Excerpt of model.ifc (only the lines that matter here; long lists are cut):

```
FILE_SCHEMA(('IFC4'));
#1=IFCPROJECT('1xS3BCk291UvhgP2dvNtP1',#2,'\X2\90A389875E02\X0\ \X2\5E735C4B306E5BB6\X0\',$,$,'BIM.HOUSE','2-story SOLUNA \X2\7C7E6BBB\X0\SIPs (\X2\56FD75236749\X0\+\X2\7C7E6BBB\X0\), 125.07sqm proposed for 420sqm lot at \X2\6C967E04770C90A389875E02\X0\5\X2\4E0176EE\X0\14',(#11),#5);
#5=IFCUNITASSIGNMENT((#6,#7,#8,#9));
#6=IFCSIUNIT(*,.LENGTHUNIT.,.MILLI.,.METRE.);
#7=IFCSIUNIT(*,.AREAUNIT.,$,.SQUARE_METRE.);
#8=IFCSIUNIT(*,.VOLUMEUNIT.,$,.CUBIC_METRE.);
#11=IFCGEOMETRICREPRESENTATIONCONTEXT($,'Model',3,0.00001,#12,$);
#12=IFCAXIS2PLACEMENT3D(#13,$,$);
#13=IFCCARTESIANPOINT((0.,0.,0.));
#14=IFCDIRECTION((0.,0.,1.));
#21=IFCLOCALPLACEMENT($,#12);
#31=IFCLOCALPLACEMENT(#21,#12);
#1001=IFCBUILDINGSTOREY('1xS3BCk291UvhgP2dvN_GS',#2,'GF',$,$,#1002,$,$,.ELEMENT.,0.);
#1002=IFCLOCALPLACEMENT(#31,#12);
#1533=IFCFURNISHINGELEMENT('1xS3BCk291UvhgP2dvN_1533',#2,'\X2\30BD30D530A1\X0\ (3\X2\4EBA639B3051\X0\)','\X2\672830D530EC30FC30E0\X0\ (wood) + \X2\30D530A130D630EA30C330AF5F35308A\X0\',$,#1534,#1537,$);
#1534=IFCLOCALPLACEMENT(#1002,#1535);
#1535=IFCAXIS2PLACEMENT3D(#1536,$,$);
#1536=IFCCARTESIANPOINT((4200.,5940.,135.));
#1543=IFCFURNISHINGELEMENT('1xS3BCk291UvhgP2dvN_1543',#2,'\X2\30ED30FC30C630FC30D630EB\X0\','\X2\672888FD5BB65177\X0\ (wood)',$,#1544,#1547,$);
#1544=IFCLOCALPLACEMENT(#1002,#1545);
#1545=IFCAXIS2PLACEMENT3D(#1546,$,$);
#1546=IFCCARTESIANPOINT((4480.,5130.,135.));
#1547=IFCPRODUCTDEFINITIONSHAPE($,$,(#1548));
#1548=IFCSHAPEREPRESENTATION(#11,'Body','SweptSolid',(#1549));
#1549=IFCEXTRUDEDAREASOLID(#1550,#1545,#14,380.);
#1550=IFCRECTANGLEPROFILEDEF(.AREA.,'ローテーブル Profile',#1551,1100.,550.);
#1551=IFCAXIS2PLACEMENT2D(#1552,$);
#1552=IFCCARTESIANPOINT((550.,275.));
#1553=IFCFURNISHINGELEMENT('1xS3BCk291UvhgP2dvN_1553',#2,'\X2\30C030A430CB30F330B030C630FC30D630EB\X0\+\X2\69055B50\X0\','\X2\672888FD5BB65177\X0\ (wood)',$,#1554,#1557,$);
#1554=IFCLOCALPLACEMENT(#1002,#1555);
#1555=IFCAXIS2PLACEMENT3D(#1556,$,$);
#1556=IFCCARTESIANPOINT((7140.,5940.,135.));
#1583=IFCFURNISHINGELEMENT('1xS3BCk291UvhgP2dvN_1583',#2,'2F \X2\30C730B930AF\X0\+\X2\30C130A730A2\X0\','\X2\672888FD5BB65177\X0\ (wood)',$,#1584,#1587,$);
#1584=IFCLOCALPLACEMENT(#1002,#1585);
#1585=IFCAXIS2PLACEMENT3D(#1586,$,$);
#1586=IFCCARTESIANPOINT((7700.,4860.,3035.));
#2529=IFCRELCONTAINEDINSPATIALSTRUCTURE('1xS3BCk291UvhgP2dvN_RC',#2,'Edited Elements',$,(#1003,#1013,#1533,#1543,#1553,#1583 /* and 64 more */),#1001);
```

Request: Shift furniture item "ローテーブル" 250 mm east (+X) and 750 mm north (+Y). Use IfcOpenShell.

```python
import ifcopenshell
import ifcopenshell.api.geometry
import ifcopenshell.util.placement
import ifcopenshell.util.unit

model = ifcopenshell.open("model.ifc")
unit_scale = ifcopenshell.util.unit.calculate_unit_scale(model)

item = model.by_guid("1xS3BCk291UvhgP2dvN_1543")
matrix = ifcopenshell.util.placement.get_local_placement(item.ObjectPlacement)
matrix[0, 3] += 0.25 / unit_scale
matrix[1, 3] += 0.75 / unit_scale
ifcopenshell.api.geometry.edit_object_placement(model, product=item, matrix=matrix, is_si=False)

print(ifcopenshell.util.placement.get_local_placement(item.ObjectPlacement).round(3) + 0.0)

model.write("model_updated.ifc")
```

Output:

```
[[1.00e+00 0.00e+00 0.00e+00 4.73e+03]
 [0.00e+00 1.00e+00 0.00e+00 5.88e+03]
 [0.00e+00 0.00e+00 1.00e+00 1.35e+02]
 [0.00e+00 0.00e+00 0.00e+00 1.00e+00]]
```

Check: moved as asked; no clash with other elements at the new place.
